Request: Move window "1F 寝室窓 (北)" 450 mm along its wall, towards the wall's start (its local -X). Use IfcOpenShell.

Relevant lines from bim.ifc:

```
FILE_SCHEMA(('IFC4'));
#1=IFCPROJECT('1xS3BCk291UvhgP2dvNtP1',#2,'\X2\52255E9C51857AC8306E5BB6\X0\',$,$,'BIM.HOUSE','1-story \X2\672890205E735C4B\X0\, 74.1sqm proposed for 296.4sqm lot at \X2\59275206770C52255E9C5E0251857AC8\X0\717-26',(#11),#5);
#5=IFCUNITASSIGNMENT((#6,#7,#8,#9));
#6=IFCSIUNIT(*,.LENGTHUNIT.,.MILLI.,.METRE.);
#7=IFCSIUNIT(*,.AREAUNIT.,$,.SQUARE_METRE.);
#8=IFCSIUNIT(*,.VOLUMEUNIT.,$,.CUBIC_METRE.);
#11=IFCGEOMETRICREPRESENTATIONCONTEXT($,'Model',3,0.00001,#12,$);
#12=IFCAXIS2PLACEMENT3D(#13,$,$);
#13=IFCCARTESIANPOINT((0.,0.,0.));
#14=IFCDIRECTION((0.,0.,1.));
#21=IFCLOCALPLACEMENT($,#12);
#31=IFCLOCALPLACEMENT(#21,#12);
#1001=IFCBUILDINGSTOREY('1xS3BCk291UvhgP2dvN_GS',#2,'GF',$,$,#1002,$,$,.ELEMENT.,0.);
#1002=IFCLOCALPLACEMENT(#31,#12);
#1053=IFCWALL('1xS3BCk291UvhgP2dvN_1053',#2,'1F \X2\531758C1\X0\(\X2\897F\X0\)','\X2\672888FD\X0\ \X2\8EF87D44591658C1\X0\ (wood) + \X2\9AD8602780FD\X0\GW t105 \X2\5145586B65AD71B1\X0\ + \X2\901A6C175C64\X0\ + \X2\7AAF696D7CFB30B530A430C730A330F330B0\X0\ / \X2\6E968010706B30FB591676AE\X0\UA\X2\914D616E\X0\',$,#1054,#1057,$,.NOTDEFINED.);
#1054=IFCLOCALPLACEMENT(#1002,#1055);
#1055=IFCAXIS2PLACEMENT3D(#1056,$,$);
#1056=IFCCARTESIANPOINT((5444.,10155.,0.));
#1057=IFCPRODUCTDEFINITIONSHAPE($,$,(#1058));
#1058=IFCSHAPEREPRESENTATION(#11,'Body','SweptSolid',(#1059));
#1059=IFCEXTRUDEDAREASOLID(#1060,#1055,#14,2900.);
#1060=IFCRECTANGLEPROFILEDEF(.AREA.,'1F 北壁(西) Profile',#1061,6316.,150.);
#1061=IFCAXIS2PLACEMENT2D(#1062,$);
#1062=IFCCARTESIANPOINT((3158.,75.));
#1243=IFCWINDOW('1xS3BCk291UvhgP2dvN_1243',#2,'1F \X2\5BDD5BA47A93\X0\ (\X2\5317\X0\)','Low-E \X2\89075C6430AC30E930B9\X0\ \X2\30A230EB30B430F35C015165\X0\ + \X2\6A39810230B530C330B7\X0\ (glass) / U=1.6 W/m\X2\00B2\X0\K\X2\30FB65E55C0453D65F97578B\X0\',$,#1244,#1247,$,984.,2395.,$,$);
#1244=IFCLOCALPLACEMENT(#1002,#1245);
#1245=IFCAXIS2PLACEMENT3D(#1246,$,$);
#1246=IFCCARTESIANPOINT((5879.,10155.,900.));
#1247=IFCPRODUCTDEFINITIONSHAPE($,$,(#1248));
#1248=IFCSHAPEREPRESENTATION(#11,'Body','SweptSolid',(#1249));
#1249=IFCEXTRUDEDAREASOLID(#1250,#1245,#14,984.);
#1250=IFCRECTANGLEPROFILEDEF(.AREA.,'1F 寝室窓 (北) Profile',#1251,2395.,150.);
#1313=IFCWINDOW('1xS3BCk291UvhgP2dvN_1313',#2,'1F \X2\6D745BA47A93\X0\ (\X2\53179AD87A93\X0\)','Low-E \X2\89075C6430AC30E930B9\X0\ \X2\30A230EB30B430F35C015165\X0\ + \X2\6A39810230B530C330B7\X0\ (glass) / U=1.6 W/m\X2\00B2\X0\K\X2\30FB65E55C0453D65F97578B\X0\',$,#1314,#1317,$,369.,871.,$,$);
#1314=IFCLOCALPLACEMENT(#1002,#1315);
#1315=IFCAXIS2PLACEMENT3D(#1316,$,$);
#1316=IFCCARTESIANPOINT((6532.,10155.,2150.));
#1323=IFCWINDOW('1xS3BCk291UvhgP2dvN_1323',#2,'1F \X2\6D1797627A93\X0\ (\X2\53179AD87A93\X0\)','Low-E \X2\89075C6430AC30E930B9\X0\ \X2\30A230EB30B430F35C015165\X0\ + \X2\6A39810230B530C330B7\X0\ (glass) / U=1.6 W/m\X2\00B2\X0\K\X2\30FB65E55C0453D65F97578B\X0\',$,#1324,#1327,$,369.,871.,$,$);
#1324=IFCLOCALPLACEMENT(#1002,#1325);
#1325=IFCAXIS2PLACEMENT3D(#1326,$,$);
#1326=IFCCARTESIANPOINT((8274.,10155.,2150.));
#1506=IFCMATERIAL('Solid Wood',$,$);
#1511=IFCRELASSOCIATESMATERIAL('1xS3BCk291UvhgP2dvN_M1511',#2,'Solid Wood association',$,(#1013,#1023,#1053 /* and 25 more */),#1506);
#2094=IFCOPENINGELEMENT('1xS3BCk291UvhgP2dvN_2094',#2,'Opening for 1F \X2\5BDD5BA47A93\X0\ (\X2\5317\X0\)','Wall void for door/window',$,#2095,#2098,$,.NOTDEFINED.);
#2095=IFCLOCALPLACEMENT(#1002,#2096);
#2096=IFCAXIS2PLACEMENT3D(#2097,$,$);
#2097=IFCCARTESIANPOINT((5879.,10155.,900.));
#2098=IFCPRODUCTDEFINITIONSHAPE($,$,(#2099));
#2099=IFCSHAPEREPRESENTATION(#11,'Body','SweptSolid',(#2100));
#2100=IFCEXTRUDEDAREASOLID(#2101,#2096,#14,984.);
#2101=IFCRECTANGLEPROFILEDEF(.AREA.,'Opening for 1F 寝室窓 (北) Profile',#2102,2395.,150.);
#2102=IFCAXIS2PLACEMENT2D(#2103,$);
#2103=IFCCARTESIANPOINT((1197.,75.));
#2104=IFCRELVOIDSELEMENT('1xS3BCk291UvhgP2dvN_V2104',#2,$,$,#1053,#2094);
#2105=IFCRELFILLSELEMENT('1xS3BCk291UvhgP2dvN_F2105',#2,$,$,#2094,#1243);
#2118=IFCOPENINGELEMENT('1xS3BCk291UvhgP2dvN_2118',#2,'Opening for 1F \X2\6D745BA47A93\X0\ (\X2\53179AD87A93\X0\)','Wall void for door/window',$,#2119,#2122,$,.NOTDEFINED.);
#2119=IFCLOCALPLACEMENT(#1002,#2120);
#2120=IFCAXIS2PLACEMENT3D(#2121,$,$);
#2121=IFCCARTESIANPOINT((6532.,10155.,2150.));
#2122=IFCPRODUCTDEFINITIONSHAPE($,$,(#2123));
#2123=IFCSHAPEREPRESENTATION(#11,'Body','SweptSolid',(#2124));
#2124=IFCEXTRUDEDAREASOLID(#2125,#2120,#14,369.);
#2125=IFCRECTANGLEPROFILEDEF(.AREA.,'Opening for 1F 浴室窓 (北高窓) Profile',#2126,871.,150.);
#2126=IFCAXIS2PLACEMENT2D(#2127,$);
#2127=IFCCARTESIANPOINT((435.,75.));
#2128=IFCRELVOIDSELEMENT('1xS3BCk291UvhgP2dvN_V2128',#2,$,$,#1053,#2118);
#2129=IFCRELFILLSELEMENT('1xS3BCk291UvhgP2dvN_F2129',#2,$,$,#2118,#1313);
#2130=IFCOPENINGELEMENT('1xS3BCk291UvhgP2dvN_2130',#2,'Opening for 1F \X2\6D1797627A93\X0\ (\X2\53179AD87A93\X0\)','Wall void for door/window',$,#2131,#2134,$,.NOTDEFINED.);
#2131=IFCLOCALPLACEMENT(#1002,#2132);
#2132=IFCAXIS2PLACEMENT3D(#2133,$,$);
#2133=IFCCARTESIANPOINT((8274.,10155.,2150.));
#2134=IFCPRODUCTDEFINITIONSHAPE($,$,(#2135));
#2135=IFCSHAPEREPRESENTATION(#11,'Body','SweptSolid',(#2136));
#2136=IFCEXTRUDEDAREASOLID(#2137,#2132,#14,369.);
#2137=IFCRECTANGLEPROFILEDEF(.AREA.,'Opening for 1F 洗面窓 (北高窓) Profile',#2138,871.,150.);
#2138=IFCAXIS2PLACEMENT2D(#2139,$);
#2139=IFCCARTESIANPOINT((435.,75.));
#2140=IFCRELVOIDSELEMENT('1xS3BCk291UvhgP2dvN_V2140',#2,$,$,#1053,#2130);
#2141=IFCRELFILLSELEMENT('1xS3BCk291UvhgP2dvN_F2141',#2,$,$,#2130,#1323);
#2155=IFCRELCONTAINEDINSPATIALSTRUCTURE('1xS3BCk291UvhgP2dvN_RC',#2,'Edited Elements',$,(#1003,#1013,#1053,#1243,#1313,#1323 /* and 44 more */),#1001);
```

```python
import ifcopenshell
import ifcopenshell.api.geometry
import ifcopenshell.util.placement
import ifcopenshell.util.unit

model = ifcopenshell.open("bim.ifc")
unit_scale = ifcopenshell.util.unit.calculate_unit_scale(model)

window = model.by_id(1243)
opening = window.FillsVoids[0].RelatingOpeningElement
wall = opening.VoidsElements[0].RelatingBuildingElement

wall_matrix = ifcopenshell.util.placement.get_local_placement(wall.ObjectPlacement)
shift = wall_matrix[:3, 0] * -0.45 / unit_scale
before = ifcopenshell.util.placement.get_local_placement(window.ObjectPlacement)[:3, 3].copy()

# The window is not placed relative to its opening, so move both.
for product in (opening, window):
    matrix = ifcopenshell.util.placement.get_local_placement(product.ObjectPlacement)
    matrix[:3, 3] += shift
    ifcopenshell.api.geometry.edit_object_placement(model, product=product, matrix=matrix, is_si=False)

after = ifcopenshell.util.placement.get_local_placement(window.ObjectPlacement)[:3, 3]
print("window moved by", (after - before).round(3) + 0.0)

model.write("bim_edited.ifc")
```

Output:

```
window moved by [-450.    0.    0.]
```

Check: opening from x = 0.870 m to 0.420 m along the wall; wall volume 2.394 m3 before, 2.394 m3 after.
